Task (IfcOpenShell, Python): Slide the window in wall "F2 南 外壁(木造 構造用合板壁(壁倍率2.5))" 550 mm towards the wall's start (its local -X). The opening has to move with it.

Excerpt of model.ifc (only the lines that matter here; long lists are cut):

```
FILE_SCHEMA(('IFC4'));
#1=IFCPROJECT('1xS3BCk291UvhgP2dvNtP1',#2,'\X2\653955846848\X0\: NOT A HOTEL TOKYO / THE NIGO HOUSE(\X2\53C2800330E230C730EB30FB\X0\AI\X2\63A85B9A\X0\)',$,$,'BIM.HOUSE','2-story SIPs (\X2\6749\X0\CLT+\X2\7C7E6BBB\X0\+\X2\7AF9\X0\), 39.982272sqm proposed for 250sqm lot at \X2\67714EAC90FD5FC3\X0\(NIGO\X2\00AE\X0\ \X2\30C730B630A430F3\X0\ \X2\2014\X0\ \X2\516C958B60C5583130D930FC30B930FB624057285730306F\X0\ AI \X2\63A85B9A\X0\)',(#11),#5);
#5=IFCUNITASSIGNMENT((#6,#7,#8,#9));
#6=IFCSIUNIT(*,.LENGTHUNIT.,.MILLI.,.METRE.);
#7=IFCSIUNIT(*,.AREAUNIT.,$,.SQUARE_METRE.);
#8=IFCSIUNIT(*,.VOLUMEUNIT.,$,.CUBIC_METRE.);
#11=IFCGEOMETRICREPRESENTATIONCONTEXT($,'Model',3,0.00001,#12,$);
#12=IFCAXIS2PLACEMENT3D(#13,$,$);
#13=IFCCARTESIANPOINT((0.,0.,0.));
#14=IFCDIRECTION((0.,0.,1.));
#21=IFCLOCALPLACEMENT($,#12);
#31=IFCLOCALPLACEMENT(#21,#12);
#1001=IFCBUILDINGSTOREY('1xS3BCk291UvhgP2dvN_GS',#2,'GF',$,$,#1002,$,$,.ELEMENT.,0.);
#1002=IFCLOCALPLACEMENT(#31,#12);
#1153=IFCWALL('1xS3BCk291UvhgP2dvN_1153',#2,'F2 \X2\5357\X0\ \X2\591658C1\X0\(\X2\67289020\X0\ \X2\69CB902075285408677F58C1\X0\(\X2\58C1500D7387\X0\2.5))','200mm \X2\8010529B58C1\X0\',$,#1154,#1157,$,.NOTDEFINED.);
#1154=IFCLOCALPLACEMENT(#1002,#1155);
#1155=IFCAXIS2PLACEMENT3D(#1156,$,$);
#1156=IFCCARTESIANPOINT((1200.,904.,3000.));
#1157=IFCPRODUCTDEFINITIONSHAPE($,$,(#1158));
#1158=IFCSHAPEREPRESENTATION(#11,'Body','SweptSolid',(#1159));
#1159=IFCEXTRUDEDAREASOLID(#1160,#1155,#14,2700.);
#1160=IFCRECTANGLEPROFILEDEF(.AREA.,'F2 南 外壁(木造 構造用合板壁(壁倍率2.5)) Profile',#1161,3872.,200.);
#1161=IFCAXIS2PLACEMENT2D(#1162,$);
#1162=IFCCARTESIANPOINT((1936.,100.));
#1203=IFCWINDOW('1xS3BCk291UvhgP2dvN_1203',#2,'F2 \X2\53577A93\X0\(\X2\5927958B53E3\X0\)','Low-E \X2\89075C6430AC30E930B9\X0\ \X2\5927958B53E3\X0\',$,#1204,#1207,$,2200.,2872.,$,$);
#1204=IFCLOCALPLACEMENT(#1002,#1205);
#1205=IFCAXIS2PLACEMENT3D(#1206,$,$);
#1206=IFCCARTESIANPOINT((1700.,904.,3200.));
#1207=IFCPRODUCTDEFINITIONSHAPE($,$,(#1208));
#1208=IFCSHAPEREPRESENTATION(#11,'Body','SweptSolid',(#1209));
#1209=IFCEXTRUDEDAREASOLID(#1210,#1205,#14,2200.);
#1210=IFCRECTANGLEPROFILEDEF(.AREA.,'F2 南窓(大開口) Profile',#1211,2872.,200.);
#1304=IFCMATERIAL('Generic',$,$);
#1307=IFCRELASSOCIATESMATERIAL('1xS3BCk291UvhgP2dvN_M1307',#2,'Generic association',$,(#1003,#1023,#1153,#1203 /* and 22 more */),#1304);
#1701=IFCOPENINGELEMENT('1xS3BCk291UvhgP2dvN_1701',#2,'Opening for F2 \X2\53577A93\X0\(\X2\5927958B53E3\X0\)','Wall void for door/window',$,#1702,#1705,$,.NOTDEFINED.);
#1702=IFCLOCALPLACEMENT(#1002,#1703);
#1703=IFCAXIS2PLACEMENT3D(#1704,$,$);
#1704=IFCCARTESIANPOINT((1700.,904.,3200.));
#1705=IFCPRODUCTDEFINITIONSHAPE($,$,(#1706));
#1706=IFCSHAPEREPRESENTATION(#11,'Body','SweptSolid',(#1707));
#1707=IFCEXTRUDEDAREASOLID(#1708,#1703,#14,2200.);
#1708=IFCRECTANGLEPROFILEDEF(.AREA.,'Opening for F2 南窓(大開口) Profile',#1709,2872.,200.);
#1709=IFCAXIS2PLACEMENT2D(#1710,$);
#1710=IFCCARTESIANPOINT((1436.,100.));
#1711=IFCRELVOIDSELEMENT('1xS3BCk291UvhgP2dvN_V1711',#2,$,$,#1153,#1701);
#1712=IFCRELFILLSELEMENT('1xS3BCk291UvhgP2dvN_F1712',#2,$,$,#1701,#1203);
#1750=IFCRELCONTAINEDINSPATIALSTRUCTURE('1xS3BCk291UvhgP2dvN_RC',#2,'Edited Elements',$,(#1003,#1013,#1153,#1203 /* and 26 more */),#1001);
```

```python
import ifcopenshell
import ifcopenshell.api.geometry
import ifcopenshell.util.placement
import ifcopenshell.util.unit

model = ifcopenshell.open("model.ifc")
unit_scale = ifcopenshell.util.unit.calculate_unit_scale(model)

window = model.by_guid("1xS3BCk291UvhgP2dvN_1203")
opening = window.FillsVoids[0].RelatingOpeningElement
wall = opening.VoidsElements[0].RelatingBuildingElement

wall_matrix = ifcopenshell.util.placement.get_local_placement(wall.ObjectPlacement)
shift = wall_matrix[:3, 0] * -0.55 / unit_scale
before = ifcopenshell.util.placement.get_local_placement(window.ObjectPlacement)[:3, 3].copy()

# The window is not placed relative to its opening, so move both.
for product in (opening, window):
    matrix = ifcopenshell.util.placement.get_local_placement(product.ObjectPlacement)
    matrix[:3, 3] += shift
    ifcopenshell.api.geometry.edit_object_placement(model, product=product, matrix=matrix, is_si=False)

after = ifcopenshell.util.placement.get_local_placement(window.ObjectPlacement)[:3, 3]
print("window moved by", (after - before).round(3) + 0.0)

model.write("model_v2.ifc")
```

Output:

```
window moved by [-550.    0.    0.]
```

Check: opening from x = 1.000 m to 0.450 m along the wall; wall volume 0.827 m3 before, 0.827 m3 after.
